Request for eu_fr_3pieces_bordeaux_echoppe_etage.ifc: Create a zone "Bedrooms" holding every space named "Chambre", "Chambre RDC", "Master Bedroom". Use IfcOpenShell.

First a look at what the model holds.

```python
import ifcopenshell

model = ifcopenshell.open("eu_fr_3pieces_bordeaux_echoppe_etage.ifc")
print(model.schema)
seen = {}
for space in model.by_type("IfcSpace"):
    seen[space.LongName] = seen.get(space.LongName, 0) + 1
for name, count in sorted(seen.items(), key=str):
    print(count, "x", name)
print("zones:", [z.Name for z in model.by_type("IfcZone")][:20])
```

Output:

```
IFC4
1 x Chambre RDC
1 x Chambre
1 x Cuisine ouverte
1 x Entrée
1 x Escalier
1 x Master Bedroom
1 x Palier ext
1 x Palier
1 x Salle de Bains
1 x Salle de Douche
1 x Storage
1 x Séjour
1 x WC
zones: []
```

```python
import ifcopenshell
import ifcopenshell.api.group
import ifcopenshell.api.root

model = ifcopenshell.open("eu_fr_3pieces_bordeaux_echoppe_etage.ifc")

names = {"Chambre", "Chambre RDC", "Master Bedroom"}
spaces = [s for s in model.by_type("IfcSpace") if s.LongName in names]

zone = ifcopenshell.api.root.create_entity(model, ifc_class="IfcZone", name="Bedrooms")
ifcopenshell.api.group.assign_group(model, products=spaces, group=zone)
print(len(spaces), "spaces in", zone.Name)

model.write("eu_fr_3pieces_bordeaux_echoppe_etage_edited.ifc")
```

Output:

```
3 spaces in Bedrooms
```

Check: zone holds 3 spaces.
